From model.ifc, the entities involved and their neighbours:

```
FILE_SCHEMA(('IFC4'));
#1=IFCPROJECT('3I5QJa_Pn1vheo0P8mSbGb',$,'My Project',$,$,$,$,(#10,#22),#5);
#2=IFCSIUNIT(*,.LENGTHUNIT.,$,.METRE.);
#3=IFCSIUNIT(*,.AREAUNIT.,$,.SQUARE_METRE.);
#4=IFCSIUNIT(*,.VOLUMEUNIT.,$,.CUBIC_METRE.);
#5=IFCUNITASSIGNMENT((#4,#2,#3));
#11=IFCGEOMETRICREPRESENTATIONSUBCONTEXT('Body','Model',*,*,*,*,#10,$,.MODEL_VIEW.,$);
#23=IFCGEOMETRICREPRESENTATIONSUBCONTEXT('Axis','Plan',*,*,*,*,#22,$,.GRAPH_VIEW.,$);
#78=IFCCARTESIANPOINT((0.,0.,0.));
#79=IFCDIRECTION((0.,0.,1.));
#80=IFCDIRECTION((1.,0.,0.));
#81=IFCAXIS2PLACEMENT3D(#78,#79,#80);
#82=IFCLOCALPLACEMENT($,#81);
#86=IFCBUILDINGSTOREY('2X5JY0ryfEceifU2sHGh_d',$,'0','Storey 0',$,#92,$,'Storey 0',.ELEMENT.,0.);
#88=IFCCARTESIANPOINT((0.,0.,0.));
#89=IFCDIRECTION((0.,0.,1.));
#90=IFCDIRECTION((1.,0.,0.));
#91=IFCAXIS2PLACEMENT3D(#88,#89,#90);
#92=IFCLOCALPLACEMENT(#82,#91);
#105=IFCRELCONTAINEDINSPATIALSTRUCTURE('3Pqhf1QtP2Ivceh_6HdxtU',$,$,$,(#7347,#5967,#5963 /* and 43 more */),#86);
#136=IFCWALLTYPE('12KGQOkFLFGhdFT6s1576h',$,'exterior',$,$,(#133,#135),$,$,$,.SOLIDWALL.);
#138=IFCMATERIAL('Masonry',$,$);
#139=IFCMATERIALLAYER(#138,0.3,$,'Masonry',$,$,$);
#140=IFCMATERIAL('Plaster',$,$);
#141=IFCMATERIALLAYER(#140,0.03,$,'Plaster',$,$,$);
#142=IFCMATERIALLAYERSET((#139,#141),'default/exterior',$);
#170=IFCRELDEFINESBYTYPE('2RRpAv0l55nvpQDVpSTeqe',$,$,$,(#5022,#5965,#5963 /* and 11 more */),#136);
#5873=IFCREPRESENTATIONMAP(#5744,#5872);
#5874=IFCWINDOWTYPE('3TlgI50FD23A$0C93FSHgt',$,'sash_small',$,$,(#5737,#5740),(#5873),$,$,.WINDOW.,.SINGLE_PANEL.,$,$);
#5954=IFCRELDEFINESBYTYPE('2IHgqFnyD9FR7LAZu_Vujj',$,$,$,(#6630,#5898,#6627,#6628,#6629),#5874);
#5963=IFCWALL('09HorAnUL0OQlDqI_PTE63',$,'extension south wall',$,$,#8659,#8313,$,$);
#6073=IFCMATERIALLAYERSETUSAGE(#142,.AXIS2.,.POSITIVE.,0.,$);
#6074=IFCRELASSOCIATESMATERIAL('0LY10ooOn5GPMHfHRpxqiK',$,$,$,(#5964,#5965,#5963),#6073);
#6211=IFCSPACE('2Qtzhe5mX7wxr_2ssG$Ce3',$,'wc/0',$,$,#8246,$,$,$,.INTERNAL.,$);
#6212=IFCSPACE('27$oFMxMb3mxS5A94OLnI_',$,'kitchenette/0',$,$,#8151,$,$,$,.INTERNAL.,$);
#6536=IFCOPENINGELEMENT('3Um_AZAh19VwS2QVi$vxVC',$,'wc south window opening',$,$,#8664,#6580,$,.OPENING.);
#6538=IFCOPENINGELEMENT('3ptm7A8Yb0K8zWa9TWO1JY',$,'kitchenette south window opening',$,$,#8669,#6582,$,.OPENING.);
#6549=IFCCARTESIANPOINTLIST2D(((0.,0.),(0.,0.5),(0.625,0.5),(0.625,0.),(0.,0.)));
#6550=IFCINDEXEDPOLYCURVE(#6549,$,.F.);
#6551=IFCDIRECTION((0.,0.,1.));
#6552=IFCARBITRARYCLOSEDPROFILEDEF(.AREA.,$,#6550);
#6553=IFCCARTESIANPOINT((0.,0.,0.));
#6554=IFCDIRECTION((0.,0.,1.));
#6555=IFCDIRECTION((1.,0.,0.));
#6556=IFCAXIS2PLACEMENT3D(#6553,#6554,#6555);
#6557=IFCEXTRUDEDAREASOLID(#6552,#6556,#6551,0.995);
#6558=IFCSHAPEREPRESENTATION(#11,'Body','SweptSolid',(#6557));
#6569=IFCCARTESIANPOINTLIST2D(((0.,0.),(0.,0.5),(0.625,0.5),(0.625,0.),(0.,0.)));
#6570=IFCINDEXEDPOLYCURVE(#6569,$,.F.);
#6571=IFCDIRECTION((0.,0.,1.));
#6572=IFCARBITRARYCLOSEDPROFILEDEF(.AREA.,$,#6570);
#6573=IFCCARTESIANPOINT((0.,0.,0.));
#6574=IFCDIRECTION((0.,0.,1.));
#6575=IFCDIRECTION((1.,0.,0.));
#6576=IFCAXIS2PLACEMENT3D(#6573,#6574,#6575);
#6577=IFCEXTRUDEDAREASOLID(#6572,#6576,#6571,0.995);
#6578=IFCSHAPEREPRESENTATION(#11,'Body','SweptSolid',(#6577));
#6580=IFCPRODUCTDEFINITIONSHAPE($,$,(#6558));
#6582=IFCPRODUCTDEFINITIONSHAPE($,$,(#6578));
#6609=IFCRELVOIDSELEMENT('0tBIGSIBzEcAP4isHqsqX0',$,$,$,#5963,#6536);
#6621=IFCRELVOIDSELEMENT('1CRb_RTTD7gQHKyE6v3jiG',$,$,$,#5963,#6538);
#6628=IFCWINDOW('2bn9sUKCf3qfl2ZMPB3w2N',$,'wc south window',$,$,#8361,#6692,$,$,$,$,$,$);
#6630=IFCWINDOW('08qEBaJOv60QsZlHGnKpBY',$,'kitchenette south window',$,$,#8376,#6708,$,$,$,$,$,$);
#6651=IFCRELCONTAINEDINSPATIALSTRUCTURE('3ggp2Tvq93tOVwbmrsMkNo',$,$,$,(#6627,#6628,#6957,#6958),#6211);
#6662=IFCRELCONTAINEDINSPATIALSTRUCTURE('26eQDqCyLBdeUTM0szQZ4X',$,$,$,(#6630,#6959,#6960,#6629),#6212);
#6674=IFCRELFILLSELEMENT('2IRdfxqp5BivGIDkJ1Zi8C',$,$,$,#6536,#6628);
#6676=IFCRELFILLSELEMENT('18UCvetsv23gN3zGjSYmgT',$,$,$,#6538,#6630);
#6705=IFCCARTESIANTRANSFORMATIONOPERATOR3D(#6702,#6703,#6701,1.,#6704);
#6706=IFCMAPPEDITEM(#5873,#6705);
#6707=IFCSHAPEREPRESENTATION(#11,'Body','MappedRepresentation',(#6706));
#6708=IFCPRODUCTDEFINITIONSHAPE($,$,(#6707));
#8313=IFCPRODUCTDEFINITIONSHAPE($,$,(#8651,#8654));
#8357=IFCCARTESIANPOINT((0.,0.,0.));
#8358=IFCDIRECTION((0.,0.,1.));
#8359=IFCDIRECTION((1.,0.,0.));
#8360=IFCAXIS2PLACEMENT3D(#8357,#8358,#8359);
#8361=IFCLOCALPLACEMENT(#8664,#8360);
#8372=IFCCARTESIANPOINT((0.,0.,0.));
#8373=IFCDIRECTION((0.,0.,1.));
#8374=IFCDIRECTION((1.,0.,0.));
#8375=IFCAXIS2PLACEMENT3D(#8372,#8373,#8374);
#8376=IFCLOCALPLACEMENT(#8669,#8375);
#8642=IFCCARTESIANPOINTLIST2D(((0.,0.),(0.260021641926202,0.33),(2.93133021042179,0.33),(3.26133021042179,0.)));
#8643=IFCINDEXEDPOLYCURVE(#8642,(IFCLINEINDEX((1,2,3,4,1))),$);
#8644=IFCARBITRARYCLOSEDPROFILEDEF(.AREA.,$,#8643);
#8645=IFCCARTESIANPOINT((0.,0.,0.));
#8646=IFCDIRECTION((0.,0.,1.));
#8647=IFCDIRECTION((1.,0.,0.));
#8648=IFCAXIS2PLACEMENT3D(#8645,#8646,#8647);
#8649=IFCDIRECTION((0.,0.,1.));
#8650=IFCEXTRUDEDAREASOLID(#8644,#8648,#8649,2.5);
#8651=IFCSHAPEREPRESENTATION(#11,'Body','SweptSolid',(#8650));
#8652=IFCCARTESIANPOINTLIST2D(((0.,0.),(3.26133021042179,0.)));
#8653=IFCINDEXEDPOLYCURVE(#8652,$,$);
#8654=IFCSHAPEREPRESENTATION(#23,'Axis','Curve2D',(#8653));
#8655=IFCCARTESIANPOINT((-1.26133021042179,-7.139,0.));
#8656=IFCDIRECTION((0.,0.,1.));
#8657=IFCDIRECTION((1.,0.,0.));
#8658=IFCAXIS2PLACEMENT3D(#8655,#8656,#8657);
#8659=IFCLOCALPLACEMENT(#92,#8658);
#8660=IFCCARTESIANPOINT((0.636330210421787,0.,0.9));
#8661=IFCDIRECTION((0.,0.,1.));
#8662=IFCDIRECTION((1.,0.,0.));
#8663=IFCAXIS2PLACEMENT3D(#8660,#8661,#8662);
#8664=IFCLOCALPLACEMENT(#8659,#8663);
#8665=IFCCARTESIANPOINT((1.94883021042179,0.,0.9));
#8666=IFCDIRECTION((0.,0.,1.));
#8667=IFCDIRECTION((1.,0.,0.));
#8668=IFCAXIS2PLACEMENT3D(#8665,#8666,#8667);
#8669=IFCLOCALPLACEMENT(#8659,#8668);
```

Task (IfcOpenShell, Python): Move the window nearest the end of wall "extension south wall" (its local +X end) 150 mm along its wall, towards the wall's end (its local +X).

```python
import ifcopenshell
import ifcopenshell.api.geometry
import ifcopenshell.util.placement
import ifcopenshell.util.unit

model = ifcopenshell.open("model.ifc")
unit_scale = ifcopenshell.util.unit.calculate_unit_scale(model)

window = model.by_guid("08qEBaJOv60QsZlHGnKpBY")
opening = window.FillsVoids[0].RelatingOpeningElement
wall = opening.VoidsElements[0].RelatingBuildingElement

wall_matrix = ifcopenshell.util.placement.get_local_placement(wall.ObjectPlacement)
shift = wall_matrix[:3, 0] * 0.15 / unit_scale
before = ifcopenshell.util.placement.get_local_placement(window.ObjectPlacement)[:3, 3].copy()

# The window is placed relative to its opening, so it follows when the opening moves.
matrix = ifcopenshell.util.placement.get_local_placement(opening.ObjectPlacement)
matrix[:3, 3] += shift
ifcopenshell.api.geometry.edit_object_placement(
    model, product=opening, matrix=matrix, is_si=False, should_transform_children=True
)

after = ifcopenshell.util.placement.get_local_placement(window.ObjectPlacement)[:3, 3]
print("window moved by", (after - before).round(3) + 0.0)

model.write("model_v2.ifc")
```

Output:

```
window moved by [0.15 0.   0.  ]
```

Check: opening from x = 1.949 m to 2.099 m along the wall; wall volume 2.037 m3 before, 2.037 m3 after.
